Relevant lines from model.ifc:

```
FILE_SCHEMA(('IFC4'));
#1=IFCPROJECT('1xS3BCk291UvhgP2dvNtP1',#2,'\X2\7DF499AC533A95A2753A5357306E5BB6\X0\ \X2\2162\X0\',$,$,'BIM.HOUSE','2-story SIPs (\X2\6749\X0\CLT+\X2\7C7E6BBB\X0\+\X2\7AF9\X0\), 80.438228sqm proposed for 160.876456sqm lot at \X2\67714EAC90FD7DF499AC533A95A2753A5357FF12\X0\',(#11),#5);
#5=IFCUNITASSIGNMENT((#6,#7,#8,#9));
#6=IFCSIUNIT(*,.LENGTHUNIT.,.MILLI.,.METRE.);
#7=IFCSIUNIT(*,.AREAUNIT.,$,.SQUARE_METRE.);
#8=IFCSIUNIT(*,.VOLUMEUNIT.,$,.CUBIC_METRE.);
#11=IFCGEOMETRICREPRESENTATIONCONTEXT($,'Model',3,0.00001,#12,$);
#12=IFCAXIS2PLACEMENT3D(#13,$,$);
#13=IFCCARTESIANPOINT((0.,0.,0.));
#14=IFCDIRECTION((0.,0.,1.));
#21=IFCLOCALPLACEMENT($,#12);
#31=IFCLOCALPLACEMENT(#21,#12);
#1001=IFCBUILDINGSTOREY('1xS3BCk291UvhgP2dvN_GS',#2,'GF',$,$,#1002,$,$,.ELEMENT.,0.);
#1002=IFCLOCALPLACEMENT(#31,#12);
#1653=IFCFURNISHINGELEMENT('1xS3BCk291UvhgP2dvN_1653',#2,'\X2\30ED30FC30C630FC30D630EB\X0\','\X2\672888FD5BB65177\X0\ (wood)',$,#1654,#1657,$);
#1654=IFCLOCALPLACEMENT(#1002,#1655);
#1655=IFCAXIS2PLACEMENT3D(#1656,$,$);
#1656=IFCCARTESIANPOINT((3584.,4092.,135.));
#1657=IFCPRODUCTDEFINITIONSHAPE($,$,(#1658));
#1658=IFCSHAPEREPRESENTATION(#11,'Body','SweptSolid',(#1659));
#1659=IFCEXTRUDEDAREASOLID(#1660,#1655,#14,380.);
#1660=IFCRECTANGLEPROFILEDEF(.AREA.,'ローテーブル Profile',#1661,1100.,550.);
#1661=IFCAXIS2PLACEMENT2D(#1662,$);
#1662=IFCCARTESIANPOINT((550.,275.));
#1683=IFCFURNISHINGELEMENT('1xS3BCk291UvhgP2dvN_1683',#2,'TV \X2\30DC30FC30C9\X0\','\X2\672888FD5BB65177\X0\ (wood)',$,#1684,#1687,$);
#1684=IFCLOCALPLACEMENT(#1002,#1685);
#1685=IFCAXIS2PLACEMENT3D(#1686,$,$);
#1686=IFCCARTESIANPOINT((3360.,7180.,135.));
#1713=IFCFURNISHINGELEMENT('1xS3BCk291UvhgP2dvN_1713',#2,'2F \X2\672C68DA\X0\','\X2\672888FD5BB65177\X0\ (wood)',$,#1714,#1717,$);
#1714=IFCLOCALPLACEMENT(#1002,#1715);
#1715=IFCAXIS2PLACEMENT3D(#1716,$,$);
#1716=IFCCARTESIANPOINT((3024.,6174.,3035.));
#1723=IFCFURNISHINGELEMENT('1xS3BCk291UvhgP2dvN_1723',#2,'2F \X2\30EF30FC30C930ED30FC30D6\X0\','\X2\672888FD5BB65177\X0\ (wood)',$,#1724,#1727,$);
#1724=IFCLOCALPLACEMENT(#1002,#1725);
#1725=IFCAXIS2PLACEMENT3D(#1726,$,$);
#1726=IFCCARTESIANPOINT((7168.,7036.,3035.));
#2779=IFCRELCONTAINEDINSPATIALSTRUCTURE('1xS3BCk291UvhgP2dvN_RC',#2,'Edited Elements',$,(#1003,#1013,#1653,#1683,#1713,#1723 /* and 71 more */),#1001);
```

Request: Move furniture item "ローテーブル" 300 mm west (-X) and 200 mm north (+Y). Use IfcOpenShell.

```python
import ifcopenshell
import ifcopenshell.api.geometry
import ifcopenshell.util.placement

model = ifcopenshell.open("model.ifc")

item = model.by_guid("1xS3BCk291UvhgP2dvN_1653")
matrix = ifcopenshell.util.placement.get_local_placement(item.ObjectPlacement)
matrix[0, 3] -= 300.0
matrix[1, 3] += 200.0
ifcopenshell.api.geometry.edit_object_placement(model, product=item, matrix=matrix, is_si=False)

print(ifcopenshell.util.placement.get_local_placement(item.ObjectPlacement).round(3) + 0.0)

model.write("model_edited.ifc")
```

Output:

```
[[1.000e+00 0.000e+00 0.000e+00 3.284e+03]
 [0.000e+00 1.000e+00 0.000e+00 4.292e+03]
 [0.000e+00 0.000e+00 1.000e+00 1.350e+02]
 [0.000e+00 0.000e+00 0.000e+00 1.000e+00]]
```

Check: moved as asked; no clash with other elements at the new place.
